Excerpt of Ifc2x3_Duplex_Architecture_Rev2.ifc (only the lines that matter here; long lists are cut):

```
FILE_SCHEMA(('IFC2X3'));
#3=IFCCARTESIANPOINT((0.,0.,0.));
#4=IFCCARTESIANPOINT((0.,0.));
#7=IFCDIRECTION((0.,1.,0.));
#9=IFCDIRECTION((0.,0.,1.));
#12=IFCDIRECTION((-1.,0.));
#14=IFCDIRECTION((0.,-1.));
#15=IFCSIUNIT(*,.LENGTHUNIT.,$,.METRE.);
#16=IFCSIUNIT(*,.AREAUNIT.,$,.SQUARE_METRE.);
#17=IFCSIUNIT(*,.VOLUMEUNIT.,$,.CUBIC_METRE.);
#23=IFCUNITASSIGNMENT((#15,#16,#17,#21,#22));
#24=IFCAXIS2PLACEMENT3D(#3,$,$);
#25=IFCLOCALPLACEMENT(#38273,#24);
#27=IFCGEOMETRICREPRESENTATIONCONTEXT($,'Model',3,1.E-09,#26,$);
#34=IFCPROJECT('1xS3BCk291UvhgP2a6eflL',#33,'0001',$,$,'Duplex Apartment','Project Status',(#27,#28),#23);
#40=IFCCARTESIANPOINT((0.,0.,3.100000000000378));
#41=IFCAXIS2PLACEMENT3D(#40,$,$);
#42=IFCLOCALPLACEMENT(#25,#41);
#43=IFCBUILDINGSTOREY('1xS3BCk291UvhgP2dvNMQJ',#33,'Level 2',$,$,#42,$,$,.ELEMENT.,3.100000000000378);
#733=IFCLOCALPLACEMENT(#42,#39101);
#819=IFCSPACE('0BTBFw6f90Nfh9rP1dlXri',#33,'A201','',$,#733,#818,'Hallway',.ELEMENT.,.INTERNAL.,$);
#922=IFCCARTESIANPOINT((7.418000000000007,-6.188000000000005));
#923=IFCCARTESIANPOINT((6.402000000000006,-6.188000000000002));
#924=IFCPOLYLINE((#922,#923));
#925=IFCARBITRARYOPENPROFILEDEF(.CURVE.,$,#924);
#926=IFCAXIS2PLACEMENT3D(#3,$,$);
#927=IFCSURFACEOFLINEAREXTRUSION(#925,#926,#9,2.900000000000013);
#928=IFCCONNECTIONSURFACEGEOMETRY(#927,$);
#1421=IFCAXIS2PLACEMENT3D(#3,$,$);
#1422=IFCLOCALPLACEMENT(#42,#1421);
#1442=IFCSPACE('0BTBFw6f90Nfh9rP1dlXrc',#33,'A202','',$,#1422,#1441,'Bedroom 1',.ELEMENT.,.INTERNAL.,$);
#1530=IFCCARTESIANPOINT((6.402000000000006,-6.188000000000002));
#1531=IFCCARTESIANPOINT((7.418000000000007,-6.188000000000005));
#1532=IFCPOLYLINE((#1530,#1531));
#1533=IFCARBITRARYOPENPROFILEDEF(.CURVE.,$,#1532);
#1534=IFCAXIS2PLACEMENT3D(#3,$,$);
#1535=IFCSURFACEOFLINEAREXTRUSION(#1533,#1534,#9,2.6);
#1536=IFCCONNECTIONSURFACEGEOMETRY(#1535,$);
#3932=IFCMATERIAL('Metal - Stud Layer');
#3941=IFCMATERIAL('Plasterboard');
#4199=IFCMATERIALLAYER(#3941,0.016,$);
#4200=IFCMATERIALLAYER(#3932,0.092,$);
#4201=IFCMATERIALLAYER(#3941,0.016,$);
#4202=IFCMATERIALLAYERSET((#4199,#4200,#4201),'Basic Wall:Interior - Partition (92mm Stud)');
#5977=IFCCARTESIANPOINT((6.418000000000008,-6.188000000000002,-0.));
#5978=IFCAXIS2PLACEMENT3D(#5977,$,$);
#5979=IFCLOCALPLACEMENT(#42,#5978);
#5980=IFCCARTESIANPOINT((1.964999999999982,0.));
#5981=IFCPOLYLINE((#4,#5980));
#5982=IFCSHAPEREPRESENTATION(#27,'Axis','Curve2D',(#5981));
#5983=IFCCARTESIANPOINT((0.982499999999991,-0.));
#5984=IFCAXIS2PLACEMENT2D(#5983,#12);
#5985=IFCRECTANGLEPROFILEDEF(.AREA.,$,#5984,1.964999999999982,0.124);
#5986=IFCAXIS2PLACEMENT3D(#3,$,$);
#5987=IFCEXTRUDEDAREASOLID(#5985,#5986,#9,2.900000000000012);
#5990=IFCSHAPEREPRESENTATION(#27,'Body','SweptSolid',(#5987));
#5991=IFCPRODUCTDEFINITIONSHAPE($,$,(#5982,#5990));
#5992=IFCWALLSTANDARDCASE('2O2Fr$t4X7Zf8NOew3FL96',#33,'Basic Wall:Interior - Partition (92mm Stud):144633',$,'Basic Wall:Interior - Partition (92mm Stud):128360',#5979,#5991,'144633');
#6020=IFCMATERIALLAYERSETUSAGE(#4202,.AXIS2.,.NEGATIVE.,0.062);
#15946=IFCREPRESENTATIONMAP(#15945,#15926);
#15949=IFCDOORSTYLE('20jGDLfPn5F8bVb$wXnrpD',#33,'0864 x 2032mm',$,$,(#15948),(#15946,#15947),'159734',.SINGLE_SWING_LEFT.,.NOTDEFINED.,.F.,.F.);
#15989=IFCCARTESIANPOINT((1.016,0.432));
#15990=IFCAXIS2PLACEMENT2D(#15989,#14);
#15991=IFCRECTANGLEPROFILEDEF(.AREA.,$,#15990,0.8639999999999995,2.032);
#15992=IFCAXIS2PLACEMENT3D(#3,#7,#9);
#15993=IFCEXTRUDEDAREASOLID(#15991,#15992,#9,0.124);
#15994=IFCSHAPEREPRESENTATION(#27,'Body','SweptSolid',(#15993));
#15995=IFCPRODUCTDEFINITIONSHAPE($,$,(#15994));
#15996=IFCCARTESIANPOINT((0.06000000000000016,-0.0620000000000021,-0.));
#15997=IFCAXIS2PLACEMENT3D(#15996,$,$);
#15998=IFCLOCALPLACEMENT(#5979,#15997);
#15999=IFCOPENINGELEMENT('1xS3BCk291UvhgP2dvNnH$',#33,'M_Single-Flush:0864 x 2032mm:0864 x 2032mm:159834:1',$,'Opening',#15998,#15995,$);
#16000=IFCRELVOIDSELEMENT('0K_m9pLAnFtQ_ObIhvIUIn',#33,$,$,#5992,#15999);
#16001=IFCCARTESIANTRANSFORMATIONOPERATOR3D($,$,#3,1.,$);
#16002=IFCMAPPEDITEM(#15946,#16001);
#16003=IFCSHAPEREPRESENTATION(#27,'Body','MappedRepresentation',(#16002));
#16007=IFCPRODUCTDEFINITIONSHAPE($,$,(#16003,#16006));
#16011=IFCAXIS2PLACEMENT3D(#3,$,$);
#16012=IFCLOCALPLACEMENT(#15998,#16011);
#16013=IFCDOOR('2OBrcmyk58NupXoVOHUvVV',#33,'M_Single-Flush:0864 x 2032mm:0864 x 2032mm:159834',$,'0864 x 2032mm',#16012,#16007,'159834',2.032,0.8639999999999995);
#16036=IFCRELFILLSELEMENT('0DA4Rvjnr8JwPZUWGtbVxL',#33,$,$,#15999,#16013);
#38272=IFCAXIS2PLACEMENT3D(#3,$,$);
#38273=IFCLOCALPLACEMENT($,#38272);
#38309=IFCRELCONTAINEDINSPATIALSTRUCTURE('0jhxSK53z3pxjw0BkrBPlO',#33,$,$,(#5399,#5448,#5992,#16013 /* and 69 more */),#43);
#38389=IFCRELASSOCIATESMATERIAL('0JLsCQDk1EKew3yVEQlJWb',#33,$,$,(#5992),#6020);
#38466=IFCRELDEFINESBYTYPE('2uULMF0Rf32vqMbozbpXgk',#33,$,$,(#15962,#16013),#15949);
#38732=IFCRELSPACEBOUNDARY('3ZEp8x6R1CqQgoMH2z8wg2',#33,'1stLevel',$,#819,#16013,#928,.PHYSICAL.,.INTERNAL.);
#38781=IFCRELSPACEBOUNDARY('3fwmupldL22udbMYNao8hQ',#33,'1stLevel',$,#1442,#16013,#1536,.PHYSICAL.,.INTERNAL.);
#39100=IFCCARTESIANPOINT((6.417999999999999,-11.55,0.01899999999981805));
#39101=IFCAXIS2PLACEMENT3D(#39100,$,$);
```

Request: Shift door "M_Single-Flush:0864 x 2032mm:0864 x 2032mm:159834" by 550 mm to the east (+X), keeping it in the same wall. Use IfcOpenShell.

```python
import numpy as np
import ifcopenshell
import ifcopenshell.api.geometry
import ifcopenshell.util.placement
import ifcopenshell.util.unit

model = ifcopenshell.open("Ifc2x3_Duplex_Architecture_Rev2.ifc")
unit_scale = ifcopenshell.util.unit.calculate_unit_scale(model)

door = model.by_id(16013)
opening = door.FillsVoids[0].RelatingOpeningElement
wall = opening.VoidsElements[0].RelatingBuildingElement

wall_matrix = ifcopenshell.util.placement.get_local_placement(wall.ObjectPlacement)
shift = wall_matrix[:3, 0] * 0.55 / unit_scale
before = ifcopenshell.util.placement.get_local_placement(door.ObjectPlacement)[:3, 3].copy()

# The door is placed relative to its opening, so it follows when the opening moves.
matrix = ifcopenshell.util.placement.get_local_placement(opening.ObjectPlacement)
matrix[:3, 3] += shift
ifcopenshell.api.geometry.edit_object_placement(
    model, product=opening, matrix=matrix, is_si=False, should_transform_children=True
)

# Space boundary surfaces are stored in each space's coordinates; move them too.
for rel in door.ProvidesBoundaries:
    if not rel.ConnectionGeometry:
        continue
    surface = rel.ConnectionGeometry.SurfaceOnRelatingElement
    space_matrix = ifcopenshell.util.placement.get_local_placement(rel.RelatingSpace.ObjectPlacement)
    point = np.array(surface.Position.Location.Coordinates) + space_matrix[:3, :3].T @ shift
    surface.Position = model.createIfcAxis2Placement3D(
        model.createIfcCartesianPoint(point.tolist()), surface.Position.Axis, surface.Position.RefDirection
    )

after = ifcopenshell.util.placement.get_local_placement(door.ObjectPlacement)[:3, 3]
print("door moved by", (after - before).round(3) + 0.0)

model.write("Ifc2x3_Duplex_Architecture_Rev2_v2.ifc")
```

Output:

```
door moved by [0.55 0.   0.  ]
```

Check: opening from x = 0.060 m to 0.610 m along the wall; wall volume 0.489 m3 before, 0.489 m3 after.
